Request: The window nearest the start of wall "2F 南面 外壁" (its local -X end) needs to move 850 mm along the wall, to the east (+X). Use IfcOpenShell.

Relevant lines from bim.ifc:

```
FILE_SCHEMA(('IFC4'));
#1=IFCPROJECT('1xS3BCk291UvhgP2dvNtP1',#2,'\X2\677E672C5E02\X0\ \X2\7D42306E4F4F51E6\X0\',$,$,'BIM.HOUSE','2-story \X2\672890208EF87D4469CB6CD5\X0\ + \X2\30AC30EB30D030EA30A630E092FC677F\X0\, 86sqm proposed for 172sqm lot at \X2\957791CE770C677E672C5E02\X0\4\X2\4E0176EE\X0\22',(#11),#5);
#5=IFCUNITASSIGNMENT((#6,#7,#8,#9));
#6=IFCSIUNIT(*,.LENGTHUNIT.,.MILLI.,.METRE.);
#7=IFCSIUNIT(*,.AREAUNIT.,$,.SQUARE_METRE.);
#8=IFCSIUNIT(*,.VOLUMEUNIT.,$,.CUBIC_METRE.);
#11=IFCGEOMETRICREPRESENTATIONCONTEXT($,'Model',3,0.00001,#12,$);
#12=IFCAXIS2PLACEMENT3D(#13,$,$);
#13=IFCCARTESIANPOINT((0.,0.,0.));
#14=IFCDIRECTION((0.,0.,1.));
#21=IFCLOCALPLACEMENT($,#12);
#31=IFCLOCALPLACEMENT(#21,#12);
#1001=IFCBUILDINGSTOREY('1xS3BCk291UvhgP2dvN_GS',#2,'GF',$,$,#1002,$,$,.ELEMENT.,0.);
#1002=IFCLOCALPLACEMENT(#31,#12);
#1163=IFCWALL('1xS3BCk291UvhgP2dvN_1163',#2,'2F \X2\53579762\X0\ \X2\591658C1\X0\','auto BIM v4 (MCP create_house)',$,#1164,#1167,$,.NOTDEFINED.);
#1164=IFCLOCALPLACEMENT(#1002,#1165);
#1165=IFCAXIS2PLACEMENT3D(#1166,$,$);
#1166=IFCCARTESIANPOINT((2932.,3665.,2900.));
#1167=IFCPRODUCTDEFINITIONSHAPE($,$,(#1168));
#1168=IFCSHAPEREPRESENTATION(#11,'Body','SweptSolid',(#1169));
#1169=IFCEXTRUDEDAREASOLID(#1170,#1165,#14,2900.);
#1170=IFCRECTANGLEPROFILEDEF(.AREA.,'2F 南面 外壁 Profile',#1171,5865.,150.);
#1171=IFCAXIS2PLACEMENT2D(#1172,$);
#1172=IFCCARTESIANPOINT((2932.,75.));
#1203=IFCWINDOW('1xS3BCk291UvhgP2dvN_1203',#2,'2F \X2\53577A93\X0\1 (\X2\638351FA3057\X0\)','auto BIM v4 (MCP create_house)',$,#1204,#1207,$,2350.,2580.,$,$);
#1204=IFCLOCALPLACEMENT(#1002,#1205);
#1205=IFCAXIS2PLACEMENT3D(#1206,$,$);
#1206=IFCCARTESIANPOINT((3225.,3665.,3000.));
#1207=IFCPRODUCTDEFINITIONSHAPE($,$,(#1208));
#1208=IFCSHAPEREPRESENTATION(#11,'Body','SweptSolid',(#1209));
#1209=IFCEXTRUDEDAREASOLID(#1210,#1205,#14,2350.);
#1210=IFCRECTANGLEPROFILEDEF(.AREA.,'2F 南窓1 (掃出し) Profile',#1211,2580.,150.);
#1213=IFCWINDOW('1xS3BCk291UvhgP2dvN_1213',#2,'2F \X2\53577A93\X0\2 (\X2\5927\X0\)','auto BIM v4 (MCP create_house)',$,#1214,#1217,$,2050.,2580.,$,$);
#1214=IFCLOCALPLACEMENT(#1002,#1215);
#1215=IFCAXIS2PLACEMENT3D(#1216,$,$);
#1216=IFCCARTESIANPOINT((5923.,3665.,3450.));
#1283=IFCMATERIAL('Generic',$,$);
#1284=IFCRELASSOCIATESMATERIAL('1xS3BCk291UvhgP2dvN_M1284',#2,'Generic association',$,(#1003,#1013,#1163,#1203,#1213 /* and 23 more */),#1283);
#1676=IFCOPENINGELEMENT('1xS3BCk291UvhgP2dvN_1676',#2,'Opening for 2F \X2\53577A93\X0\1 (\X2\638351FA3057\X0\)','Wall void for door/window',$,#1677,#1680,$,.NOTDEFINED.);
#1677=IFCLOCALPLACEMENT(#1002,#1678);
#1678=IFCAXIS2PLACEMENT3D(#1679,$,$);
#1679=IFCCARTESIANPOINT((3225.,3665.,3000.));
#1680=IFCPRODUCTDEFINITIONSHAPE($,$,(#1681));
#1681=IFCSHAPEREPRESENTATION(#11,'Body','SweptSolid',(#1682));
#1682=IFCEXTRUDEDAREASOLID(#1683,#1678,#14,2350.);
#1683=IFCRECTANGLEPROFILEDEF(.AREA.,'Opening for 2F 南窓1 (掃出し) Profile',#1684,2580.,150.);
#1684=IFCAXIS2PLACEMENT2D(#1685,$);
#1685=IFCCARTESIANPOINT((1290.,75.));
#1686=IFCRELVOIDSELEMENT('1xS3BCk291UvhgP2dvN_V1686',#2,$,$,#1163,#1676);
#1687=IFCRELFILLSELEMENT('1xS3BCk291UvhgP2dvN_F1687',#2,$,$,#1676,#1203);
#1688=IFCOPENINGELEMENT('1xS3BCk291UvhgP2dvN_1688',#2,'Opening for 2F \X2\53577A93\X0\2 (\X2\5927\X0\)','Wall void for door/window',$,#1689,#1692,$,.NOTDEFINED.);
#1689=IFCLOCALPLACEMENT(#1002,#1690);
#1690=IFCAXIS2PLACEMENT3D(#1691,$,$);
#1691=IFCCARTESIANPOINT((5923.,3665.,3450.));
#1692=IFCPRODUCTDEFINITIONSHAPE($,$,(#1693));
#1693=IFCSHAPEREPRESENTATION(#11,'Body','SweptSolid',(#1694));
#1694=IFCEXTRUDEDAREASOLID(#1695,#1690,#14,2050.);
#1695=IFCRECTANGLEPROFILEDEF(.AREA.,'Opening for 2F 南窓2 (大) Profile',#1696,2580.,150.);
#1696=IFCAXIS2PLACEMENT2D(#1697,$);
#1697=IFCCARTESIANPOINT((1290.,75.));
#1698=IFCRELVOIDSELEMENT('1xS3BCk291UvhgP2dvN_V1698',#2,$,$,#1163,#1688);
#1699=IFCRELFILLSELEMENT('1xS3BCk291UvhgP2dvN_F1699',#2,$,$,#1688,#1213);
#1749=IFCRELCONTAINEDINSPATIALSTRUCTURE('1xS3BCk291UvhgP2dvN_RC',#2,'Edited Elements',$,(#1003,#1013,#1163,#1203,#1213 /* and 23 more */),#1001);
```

```python
import ifcopenshell
import ifcopenshell.api.geometry
import ifcopenshell.util.placement
import ifcopenshell.util.unit

model = ifcopenshell.open("bim.ifc")
unit_scale = ifcopenshell.util.unit.calculate_unit_scale(model)

window = model.by_id(1203)
opening = window.FillsVoids[0].RelatingOpeningElement
wall = opening.VoidsElements[0].RelatingBuildingElement

wall_matrix = ifcopenshell.util.placement.get_local_placement(wall.ObjectPlacement)
shift = wall_matrix[:3, 0] * 0.85 / unit_scale
before = ifcopenshell.util.placement.get_local_placement(window.ObjectPlacement)[:3, 3].copy()

# The window is not placed relative to its opening, so move both.
for product in (opening, window):
    matrix = ifcopenshell.util.placement.get_local_placement(product.ObjectPlacement)
    matrix[:3, 3] += shift
    ifcopenshell.api.geometry.edit_object_placement(model, product=product, matrix=matrix, is_si=False)

after = ifcopenshell.util.placement.get_local_placement(window.ObjectPlacement)[:3, 3]
print("window moved by", (after - before).round(3) + 0.0)

model.write("bim_edited.ifc")
```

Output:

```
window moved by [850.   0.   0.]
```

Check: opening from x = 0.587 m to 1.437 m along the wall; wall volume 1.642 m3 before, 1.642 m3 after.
